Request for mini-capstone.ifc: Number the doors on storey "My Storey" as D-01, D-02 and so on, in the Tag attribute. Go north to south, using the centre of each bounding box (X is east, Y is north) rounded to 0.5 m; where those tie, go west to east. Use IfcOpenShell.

First a look at what the model holds.

```python
import ifcopenshell
import ifcopenshell.util.element
import ifcopenshell.util.placement

model = ifcopenshell.open("mini-capstone.ifc")
print(model.schema)
storey = next(s for s in model.by_type("IfcBuildingStorey") if s.Name == "My Storey")
doors = [e for e in ifcopenshell.util.element.get_decomposition(storey) if e.is_a("IfcDoor")]
for e in sorted(doors, key=lambda e: e.id()):
    origin = ifcopenshell.util.placement.get_local_placement(e.ObjectPlacement)[:3, 3]
    print(e.id(), e.Tag, e.Name, origin.round(2) + 0.0, sep=" | ")
```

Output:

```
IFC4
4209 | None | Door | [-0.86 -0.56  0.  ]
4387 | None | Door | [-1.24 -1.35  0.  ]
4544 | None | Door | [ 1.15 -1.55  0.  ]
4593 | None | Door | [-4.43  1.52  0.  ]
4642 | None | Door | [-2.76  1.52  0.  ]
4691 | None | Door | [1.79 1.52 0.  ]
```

```python
import ifcopenshell
import ifcopenshell.geom
import ifcopenshell.util.element
import ifcopenshell.util.shape

model = ifcopenshell.open("mini-capstone.ifc")
settings = ifcopenshell.geom.settings()
settings.set("use-world-coords", True)


def centre(element):
    shape = ifcopenshell.geom.create_shape(settings, element)
    return ifcopenshell.util.shape.get_bbox_centroid(shape.geometry)


storey = next(s for s in model.by_type("IfcBuildingStorey") if s.Name == "My Storey")
doors = [e for e in ifcopenshell.util.element.get_decomposition(storey) if e.is_a("IfcDoor")]

# Insertion points can sit at a corner or the storey origin, so sort by the geometry (in metres).
centres = {e: centre(e) for e in doors}
doors.sort(key=lambda e: (-round(centres[e][1] / 0.5), centres[e][0]))

for i, e in enumerate(doors, start=1):
    number = f"D-{i:02d}"
    e.Tag = number
    print(e.id(), number)

model.write("mini-capstone-out.ifc")
```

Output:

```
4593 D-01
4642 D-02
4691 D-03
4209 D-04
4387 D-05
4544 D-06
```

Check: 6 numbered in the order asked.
